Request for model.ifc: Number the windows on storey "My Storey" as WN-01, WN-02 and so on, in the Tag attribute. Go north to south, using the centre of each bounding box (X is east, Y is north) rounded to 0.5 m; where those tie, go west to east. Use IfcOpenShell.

First a look at what the model holds.

```python
import ifcopenshell
import ifcopenshell.util.element
import ifcopenshell.util.placement

model = ifcopenshell.open("model.ifc")
print(model.schema)
storey = next(s for s in model.by_type("IfcBuildingStorey") if s.Name == "My Storey")
windows = [e for e in ifcopenshell.util.element.get_decomposition(storey) if e.is_a("IfcWindow")]
for e in sorted(windows, key=lambda e: e.id()):
    origin = ifcopenshell.util.placement.get_local_placement(e.ObjectPlacement)[:3, 3]
    print(e.id(), e.Tag, e.Name, origin.round(2) + 0.0, sep=" | ")
```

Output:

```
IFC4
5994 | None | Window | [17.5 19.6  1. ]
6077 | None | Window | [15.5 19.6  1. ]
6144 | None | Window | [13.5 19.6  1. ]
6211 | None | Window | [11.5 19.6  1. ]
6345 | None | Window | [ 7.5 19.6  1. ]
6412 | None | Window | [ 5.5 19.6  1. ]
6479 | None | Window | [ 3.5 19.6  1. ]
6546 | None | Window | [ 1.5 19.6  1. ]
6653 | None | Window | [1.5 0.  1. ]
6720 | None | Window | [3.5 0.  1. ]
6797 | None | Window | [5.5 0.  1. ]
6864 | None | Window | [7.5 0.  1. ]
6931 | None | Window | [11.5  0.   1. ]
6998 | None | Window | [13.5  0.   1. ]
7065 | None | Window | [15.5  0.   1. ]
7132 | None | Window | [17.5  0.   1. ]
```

```python
import ifcopenshell
import ifcopenshell.geom
import ifcopenshell.util.element
import ifcopenshell.util.shape

model = ifcopenshell.open("model.ifc")
settings = ifcopenshell.geom.settings()
settings.set("use-world-coords", True)


def centre(element):
    shape = ifcopenshell.geom.create_shape(settings, element)
    return ifcopenshell.util.shape.get_bbox_centroid(shape.geometry)


storey = next(s for s in model.by_type("IfcBuildingStorey") if s.Name == "My Storey")
windows = [e for e in ifcopenshell.util.element.get_decomposition(storey) if e.is_a("IfcWindow")]

# Insertion points can sit at a corner or the storey origin, so sort by the geometry (in metres).
centres = {e: centre(e) for e in windows}
windows.sort(key=lambda e: (-round(centres[e][1] / 0.5), centres[e][0]))

for i, e in enumerate(windows, start=1):
    number = f"WN-{i:02d}"
    e.Tag = number
    print(e.id(), number)

model.write("model_v2.ifc")
```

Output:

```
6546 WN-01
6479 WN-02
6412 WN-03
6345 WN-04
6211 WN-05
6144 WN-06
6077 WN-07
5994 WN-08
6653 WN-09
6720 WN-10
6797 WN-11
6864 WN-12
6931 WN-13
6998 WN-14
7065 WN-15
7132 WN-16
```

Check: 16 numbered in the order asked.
